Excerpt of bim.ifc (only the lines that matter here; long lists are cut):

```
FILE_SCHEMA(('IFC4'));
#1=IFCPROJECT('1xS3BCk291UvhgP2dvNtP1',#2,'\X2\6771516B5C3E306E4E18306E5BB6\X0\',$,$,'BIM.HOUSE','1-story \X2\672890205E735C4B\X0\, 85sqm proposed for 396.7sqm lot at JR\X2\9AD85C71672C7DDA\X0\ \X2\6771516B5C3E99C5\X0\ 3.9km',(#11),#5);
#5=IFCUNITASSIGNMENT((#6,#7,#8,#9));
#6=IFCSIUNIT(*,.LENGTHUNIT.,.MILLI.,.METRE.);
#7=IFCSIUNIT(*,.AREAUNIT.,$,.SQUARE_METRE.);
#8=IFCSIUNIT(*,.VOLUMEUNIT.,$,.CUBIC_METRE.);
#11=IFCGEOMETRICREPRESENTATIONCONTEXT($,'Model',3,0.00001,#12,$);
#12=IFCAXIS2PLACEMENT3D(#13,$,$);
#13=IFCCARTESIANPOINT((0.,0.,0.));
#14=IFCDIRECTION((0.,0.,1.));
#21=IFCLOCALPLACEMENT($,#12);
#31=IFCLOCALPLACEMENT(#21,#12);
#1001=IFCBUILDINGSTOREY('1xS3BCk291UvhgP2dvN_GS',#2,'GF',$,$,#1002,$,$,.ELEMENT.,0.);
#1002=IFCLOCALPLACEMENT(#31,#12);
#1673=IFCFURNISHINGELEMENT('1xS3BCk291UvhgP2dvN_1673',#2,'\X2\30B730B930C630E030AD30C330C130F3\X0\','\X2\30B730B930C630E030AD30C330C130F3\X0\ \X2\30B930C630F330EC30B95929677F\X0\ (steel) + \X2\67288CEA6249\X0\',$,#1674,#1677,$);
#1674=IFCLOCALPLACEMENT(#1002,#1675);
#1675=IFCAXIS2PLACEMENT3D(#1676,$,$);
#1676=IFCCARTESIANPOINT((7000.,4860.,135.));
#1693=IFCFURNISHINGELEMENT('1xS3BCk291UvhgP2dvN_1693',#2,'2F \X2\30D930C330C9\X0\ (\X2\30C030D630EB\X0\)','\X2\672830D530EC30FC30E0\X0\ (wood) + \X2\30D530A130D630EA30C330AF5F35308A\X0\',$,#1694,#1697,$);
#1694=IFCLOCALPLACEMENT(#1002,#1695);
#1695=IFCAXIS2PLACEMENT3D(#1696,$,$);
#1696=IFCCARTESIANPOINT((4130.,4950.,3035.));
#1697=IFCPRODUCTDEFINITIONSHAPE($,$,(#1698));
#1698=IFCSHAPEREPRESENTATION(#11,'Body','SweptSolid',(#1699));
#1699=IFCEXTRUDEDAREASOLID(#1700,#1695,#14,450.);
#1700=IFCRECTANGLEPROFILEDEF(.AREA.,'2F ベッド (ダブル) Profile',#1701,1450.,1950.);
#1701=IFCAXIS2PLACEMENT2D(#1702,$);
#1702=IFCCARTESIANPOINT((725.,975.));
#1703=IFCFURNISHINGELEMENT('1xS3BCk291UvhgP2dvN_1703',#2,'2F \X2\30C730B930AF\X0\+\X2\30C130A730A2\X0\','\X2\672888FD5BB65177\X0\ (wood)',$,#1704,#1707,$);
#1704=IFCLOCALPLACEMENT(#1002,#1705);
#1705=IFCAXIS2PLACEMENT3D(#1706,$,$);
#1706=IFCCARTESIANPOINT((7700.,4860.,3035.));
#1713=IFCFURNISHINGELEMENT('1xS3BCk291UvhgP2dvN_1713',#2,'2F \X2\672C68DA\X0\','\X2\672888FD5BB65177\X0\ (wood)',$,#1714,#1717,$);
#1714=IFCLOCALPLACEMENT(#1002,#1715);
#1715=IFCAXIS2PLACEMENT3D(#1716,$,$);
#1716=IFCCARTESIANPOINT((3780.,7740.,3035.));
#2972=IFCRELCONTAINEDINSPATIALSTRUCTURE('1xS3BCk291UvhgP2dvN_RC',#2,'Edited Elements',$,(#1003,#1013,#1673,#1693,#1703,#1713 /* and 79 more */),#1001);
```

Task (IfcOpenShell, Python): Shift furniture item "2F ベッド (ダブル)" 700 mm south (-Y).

```python
import ifcopenshell
import ifcopenshell.api.geometry
import ifcopenshell.util.placement
import ifcopenshell.util.unit

model = ifcopenshell.open("bim.ifc")
unit_scale = ifcopenshell.util.unit.calculate_unit_scale(model)

item = model.by_guid("1xS3BCk291UvhgP2dvN_1693")
matrix = ifcopenshell.util.placement.get_local_placement(item.ObjectPlacement)
matrix[1, 3] -= 0.7 / unit_scale
ifcopenshell.api.geometry.edit_object_placement(model, product=item, matrix=matrix, is_si=False)

print(ifcopenshell.util.placement.get_local_placement(item.ObjectPlacement).round(3) + 0.0)

model.write("bim_v2.ifc")
```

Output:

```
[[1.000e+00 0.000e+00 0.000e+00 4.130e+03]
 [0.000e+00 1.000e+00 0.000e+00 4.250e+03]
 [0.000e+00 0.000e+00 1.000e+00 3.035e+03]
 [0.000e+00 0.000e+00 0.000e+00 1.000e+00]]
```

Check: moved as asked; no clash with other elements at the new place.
